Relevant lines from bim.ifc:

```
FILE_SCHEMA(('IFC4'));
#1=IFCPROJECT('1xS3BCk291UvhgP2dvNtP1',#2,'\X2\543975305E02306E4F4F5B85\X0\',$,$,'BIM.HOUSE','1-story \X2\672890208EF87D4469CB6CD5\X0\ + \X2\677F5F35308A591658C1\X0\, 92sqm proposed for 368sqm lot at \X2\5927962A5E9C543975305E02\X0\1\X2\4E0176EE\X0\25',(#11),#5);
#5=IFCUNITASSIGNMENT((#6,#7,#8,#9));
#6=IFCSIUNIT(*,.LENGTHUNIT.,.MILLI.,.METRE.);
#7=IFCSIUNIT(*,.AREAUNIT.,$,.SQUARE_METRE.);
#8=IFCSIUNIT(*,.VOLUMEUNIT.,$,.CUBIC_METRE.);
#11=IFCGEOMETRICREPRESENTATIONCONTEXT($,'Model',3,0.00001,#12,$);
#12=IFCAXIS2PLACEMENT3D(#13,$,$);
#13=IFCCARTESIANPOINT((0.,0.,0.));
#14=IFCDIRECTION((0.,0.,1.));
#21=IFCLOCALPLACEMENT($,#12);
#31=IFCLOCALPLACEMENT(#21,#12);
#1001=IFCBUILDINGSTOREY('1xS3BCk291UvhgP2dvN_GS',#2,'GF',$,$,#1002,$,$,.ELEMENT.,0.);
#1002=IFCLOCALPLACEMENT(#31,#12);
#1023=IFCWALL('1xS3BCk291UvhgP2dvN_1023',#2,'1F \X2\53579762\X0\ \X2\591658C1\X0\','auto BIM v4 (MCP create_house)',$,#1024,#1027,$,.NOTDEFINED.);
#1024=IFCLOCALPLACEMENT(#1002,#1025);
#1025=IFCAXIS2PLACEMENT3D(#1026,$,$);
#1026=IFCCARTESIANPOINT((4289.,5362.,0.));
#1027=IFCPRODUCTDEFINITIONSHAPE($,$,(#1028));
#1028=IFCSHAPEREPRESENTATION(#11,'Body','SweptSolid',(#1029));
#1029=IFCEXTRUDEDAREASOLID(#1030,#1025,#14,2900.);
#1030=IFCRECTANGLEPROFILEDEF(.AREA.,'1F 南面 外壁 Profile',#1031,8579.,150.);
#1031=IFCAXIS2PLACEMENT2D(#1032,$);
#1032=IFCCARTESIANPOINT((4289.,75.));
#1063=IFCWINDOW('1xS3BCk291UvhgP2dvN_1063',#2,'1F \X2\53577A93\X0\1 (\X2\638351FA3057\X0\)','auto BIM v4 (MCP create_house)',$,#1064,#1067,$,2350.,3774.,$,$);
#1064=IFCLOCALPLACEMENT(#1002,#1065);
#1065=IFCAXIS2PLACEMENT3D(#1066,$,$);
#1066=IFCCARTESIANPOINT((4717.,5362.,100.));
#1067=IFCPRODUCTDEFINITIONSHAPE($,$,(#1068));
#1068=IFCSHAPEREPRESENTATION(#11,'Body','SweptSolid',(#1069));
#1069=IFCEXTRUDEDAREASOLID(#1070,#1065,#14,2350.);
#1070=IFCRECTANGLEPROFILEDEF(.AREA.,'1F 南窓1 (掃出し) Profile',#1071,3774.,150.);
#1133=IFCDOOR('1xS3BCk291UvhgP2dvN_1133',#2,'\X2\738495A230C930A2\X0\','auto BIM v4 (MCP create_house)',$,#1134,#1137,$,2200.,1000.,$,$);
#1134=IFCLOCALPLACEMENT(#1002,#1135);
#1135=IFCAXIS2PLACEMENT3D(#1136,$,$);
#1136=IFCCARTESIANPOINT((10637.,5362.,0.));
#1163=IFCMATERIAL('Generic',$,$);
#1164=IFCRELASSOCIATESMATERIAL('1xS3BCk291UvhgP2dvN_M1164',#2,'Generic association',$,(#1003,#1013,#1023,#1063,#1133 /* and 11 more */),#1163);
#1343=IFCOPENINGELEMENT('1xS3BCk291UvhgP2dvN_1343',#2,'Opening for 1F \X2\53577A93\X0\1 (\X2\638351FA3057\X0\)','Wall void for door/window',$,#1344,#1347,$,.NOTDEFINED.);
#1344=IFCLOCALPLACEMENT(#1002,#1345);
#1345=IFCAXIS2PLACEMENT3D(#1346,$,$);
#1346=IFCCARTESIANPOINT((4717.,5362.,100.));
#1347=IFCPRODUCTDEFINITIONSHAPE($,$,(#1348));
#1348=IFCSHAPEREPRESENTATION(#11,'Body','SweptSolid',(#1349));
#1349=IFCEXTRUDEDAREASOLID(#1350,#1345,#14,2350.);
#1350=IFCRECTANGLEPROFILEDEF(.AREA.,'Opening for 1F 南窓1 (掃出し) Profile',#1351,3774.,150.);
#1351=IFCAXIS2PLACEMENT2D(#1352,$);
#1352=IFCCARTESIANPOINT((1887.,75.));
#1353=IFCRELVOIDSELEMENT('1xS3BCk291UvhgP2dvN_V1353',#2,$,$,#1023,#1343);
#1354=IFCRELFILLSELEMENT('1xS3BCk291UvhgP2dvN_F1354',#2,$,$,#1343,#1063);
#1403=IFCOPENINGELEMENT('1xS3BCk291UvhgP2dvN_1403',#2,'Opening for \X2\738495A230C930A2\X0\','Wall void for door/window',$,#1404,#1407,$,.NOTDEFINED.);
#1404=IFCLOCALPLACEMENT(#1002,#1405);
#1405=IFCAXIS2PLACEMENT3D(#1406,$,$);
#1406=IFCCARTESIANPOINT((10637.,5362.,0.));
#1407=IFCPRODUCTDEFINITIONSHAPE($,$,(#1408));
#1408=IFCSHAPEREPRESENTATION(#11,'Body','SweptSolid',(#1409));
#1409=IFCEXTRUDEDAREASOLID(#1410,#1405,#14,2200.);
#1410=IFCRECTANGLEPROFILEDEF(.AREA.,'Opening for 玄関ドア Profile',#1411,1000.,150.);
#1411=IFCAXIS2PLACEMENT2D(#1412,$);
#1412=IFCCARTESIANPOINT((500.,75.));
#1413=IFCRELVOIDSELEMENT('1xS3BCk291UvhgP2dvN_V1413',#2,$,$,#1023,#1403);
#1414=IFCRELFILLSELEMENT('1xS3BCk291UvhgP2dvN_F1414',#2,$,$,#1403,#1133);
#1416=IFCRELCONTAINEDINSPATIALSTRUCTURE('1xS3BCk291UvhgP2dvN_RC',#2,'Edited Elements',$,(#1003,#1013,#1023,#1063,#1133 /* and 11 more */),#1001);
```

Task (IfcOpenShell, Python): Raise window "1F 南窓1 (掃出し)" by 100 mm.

```python
import numpy as np
import ifcopenshell
import ifcopenshell.api.geometry
import ifcopenshell.util.placement
import ifcopenshell.util.unit

model = ifcopenshell.open("bim.ifc")
unit_scale = ifcopenshell.util.unit.calculate_unit_scale(model)

window = model.by_guid("1xS3BCk291UvhgP2dvN_1063")
opening = window.FillsVoids[0].RelatingOpeningElement
dz = 0.1 / unit_scale

shift = np.array([0.0, 0.0, dz])
# The window is not placed relative to its opening, so move both.
for product in (opening, window):
    matrix = ifcopenshell.util.placement.get_local_placement(product.ObjectPlacement)
    matrix[:3, 3] += shift
    ifcopenshell.api.geometry.edit_object_placement(model, product=product, matrix=matrix, is_si=False)

print(f"moved by {dz * unit_scale:+.3f} m")

model.write("bim_edited.ifc")
```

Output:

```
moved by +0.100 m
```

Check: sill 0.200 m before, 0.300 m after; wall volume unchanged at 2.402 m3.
